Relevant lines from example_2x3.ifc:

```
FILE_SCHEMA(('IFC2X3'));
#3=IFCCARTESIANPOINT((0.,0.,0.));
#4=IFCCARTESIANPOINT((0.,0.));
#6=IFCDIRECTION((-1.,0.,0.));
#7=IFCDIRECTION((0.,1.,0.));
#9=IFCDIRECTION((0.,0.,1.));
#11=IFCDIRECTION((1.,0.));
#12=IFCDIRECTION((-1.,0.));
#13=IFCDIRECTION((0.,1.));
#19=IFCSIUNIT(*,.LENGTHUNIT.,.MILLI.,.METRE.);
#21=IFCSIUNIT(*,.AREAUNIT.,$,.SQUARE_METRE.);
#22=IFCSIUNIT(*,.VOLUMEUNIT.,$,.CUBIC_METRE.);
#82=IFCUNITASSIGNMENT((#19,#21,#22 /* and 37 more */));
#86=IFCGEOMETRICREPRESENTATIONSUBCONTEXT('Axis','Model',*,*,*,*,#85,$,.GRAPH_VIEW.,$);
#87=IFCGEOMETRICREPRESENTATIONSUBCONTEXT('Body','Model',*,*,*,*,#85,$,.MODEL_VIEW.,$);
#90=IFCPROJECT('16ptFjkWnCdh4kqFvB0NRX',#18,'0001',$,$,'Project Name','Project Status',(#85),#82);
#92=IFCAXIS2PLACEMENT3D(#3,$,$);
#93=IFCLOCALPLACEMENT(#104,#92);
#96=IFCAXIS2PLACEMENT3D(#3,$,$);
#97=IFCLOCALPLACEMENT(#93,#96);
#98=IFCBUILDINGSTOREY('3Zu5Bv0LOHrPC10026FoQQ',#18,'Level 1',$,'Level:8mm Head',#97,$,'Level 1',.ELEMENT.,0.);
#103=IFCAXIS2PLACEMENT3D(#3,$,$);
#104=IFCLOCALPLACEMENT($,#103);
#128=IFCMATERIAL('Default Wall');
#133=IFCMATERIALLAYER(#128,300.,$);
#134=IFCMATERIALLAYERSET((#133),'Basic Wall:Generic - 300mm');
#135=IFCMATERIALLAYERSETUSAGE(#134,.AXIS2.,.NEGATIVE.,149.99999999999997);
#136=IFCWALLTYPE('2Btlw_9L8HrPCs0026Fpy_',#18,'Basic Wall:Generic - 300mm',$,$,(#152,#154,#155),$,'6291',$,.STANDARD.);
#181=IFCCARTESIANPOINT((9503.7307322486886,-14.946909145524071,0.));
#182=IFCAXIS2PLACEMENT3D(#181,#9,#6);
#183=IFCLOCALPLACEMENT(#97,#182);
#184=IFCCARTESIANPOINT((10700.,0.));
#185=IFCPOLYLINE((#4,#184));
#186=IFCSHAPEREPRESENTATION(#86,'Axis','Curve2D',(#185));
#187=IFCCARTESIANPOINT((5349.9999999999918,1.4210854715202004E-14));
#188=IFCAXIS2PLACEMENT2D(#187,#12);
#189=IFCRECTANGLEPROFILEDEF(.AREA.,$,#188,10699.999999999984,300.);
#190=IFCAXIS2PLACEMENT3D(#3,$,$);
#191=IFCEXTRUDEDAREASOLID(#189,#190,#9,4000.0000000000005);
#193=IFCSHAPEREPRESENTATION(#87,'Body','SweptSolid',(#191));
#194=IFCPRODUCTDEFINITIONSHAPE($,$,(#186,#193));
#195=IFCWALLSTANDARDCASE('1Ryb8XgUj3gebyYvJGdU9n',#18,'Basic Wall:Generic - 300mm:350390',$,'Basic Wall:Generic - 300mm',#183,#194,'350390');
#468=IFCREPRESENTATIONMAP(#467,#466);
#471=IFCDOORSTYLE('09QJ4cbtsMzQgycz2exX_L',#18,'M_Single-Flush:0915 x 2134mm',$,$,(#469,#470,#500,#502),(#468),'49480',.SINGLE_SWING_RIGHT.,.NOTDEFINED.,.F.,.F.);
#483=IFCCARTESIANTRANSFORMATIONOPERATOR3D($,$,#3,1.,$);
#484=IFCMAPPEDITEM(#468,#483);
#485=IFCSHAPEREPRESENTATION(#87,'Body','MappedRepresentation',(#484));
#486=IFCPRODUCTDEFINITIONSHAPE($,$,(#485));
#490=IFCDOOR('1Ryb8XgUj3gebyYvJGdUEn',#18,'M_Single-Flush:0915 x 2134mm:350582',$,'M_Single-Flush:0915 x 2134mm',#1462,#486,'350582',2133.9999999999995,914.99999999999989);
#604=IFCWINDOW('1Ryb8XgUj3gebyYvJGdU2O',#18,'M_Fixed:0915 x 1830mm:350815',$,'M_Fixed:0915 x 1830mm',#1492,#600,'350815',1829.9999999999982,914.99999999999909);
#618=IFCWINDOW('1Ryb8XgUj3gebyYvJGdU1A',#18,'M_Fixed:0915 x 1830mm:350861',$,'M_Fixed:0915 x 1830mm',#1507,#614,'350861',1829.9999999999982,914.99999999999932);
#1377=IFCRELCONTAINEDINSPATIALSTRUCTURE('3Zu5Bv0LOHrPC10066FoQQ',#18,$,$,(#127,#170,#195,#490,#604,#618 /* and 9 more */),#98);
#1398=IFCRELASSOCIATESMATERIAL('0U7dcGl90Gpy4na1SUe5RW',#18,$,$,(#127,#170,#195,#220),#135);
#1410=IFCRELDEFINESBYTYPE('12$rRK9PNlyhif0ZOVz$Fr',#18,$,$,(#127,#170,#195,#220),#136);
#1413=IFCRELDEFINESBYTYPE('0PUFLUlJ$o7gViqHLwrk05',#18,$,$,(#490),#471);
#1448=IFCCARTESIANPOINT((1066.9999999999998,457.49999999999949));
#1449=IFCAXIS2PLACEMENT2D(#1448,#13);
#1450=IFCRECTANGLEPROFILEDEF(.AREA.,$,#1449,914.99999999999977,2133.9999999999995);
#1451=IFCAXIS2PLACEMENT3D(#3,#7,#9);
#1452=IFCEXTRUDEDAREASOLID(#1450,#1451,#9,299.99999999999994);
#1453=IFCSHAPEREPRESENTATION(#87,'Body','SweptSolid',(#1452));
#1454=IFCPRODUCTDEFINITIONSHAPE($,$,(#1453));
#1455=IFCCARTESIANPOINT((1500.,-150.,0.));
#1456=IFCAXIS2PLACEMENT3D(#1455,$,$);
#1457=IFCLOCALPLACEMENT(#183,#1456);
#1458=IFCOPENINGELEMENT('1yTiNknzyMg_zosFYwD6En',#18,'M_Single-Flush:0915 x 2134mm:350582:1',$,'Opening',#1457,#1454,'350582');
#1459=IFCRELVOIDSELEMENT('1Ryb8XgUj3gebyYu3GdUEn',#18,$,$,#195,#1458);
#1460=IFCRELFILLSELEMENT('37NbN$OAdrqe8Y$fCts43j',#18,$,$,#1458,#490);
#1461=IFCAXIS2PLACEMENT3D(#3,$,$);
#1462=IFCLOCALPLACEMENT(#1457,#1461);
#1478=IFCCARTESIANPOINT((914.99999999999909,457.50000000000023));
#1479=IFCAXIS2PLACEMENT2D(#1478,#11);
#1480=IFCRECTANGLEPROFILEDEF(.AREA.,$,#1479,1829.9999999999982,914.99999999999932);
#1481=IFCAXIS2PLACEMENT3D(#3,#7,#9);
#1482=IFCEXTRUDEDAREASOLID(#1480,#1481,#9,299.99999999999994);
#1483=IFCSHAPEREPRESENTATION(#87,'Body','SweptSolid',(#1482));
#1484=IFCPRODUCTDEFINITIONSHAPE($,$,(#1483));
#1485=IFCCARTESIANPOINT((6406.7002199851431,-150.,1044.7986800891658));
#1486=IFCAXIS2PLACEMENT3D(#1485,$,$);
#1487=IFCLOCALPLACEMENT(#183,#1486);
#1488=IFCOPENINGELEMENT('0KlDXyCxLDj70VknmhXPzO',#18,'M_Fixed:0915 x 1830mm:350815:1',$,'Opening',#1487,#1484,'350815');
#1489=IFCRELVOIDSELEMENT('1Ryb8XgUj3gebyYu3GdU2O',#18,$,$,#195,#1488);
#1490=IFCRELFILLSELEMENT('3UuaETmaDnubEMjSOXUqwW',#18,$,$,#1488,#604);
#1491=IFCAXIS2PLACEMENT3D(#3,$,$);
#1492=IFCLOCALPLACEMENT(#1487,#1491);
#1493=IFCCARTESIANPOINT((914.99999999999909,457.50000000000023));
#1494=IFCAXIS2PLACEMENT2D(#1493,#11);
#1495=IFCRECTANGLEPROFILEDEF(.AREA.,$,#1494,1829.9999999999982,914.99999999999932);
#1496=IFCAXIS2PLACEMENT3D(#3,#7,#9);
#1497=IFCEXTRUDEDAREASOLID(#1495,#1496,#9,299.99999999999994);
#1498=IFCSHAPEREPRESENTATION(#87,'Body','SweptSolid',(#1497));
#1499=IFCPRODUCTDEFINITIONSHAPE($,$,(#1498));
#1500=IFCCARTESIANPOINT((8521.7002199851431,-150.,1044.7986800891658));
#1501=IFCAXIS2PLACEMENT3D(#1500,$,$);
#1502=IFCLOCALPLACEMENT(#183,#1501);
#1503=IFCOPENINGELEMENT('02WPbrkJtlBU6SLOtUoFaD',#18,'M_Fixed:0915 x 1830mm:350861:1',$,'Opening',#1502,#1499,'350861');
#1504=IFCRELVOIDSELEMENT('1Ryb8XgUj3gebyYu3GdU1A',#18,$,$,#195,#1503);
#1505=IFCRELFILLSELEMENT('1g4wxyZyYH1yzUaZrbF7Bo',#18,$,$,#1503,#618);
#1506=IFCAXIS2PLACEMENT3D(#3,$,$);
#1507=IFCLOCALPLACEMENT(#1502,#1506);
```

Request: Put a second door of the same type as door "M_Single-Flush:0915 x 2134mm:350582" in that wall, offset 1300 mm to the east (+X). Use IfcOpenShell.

```python
import ifcopenshell
import ifcopenshell.api.feature
import ifcopenshell.api.geometry
import ifcopenshell.api.root
import ifcopenshell.geom
import ifcopenshell.util.element
import ifcopenshell.util.placement
import ifcopenshell.util.shape
import ifcopenshell.util.unit

model = ifcopenshell.open("example_2x3.ifc")
unit_scale = ifcopenshell.util.unit.calculate_unit_scale(model)
settings = ifcopenshell.geom.settings()


def volume(element):
    """Net volume in cubic metres, openings subtracted."""
    shape = ifcopenshell.geom.create_shape(settings, element)
    return ifcopenshell.util.shape.get_volume(shape.geometry)


def reuse_history(source, copy):
    """copy_class also copies each property set's owner history, people and application; keep the originals."""
    for rel in copy.IsDefinedBy:
        if rel.is_a("IfcRelDefinesByProperties") and (history := rel.RelatingPropertyDefinition.OwnerHistory):
            rel.RelatingPropertyDefinition.OwnerHistory = source.OwnerHistory
            ifcopenshell.util.element.remove_deep2(model, history)


door = model.by_guid("1Ryb8XgUj3gebyYvJGdUEn")
opening = door.FillsVoids[0].RelatingOpeningElement
wall = opening.VoidsElements[0].RelatingBuildingElement
before = volume(wall)
shift = ifcopenshell.util.placement.get_local_placement(wall.ObjectPlacement)[:3, 0] * -1.3 / unit_scale

# copy_class copies the void relationship, type, container and properties, but no geometry.
new_opening = ifcopenshell.api.root.copy_class(model, product=opening)
new_opening.Representation = ifcopenshell.util.element.copy_deep(
    model, opening.Representation, exclude=["IfcGeometricRepresentationContext", "IfcRepresentationMap"]
)
new_opening.Name = "M_Single-Flush:0915 x 2134mm"
new_opening.Tag = None
new_door = ifcopenshell.api.root.copy_class(model, product=door)
new_door.Representation = ifcopenshell.util.element.copy_deep(
    model, door.Representation, exclude=["IfcGeometricRepresentationContext", "IfcRepresentationMap"]
)
new_door.Name = "M_Single-Flush:0915 x 2134mm"
new_door.Tag = None
reuse_history(door, new_door)
fills = ifcopenshell.api.feature.add_filling(model, opening=new_opening, element=new_door)
fills.OwnerHistory = new_door.OwnerHistory  # required in IFC2X3

for old, new in ((opening, new_opening), (door, new_door)):
    matrix = ifcopenshell.util.placement.get_local_placement(old.ObjectPlacement)
    matrix[:3, 3] += shift
    ifcopenshell.api.geometry.edit_object_placement(model, product=new, matrix=matrix, is_si=False)

after = volume(wall)

print(f"wall volume {before:.3f} -> {after:.3f} m3")

model.write("example_2x3_v2.ifc")
```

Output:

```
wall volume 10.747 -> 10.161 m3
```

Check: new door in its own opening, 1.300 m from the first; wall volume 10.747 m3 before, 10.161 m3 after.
